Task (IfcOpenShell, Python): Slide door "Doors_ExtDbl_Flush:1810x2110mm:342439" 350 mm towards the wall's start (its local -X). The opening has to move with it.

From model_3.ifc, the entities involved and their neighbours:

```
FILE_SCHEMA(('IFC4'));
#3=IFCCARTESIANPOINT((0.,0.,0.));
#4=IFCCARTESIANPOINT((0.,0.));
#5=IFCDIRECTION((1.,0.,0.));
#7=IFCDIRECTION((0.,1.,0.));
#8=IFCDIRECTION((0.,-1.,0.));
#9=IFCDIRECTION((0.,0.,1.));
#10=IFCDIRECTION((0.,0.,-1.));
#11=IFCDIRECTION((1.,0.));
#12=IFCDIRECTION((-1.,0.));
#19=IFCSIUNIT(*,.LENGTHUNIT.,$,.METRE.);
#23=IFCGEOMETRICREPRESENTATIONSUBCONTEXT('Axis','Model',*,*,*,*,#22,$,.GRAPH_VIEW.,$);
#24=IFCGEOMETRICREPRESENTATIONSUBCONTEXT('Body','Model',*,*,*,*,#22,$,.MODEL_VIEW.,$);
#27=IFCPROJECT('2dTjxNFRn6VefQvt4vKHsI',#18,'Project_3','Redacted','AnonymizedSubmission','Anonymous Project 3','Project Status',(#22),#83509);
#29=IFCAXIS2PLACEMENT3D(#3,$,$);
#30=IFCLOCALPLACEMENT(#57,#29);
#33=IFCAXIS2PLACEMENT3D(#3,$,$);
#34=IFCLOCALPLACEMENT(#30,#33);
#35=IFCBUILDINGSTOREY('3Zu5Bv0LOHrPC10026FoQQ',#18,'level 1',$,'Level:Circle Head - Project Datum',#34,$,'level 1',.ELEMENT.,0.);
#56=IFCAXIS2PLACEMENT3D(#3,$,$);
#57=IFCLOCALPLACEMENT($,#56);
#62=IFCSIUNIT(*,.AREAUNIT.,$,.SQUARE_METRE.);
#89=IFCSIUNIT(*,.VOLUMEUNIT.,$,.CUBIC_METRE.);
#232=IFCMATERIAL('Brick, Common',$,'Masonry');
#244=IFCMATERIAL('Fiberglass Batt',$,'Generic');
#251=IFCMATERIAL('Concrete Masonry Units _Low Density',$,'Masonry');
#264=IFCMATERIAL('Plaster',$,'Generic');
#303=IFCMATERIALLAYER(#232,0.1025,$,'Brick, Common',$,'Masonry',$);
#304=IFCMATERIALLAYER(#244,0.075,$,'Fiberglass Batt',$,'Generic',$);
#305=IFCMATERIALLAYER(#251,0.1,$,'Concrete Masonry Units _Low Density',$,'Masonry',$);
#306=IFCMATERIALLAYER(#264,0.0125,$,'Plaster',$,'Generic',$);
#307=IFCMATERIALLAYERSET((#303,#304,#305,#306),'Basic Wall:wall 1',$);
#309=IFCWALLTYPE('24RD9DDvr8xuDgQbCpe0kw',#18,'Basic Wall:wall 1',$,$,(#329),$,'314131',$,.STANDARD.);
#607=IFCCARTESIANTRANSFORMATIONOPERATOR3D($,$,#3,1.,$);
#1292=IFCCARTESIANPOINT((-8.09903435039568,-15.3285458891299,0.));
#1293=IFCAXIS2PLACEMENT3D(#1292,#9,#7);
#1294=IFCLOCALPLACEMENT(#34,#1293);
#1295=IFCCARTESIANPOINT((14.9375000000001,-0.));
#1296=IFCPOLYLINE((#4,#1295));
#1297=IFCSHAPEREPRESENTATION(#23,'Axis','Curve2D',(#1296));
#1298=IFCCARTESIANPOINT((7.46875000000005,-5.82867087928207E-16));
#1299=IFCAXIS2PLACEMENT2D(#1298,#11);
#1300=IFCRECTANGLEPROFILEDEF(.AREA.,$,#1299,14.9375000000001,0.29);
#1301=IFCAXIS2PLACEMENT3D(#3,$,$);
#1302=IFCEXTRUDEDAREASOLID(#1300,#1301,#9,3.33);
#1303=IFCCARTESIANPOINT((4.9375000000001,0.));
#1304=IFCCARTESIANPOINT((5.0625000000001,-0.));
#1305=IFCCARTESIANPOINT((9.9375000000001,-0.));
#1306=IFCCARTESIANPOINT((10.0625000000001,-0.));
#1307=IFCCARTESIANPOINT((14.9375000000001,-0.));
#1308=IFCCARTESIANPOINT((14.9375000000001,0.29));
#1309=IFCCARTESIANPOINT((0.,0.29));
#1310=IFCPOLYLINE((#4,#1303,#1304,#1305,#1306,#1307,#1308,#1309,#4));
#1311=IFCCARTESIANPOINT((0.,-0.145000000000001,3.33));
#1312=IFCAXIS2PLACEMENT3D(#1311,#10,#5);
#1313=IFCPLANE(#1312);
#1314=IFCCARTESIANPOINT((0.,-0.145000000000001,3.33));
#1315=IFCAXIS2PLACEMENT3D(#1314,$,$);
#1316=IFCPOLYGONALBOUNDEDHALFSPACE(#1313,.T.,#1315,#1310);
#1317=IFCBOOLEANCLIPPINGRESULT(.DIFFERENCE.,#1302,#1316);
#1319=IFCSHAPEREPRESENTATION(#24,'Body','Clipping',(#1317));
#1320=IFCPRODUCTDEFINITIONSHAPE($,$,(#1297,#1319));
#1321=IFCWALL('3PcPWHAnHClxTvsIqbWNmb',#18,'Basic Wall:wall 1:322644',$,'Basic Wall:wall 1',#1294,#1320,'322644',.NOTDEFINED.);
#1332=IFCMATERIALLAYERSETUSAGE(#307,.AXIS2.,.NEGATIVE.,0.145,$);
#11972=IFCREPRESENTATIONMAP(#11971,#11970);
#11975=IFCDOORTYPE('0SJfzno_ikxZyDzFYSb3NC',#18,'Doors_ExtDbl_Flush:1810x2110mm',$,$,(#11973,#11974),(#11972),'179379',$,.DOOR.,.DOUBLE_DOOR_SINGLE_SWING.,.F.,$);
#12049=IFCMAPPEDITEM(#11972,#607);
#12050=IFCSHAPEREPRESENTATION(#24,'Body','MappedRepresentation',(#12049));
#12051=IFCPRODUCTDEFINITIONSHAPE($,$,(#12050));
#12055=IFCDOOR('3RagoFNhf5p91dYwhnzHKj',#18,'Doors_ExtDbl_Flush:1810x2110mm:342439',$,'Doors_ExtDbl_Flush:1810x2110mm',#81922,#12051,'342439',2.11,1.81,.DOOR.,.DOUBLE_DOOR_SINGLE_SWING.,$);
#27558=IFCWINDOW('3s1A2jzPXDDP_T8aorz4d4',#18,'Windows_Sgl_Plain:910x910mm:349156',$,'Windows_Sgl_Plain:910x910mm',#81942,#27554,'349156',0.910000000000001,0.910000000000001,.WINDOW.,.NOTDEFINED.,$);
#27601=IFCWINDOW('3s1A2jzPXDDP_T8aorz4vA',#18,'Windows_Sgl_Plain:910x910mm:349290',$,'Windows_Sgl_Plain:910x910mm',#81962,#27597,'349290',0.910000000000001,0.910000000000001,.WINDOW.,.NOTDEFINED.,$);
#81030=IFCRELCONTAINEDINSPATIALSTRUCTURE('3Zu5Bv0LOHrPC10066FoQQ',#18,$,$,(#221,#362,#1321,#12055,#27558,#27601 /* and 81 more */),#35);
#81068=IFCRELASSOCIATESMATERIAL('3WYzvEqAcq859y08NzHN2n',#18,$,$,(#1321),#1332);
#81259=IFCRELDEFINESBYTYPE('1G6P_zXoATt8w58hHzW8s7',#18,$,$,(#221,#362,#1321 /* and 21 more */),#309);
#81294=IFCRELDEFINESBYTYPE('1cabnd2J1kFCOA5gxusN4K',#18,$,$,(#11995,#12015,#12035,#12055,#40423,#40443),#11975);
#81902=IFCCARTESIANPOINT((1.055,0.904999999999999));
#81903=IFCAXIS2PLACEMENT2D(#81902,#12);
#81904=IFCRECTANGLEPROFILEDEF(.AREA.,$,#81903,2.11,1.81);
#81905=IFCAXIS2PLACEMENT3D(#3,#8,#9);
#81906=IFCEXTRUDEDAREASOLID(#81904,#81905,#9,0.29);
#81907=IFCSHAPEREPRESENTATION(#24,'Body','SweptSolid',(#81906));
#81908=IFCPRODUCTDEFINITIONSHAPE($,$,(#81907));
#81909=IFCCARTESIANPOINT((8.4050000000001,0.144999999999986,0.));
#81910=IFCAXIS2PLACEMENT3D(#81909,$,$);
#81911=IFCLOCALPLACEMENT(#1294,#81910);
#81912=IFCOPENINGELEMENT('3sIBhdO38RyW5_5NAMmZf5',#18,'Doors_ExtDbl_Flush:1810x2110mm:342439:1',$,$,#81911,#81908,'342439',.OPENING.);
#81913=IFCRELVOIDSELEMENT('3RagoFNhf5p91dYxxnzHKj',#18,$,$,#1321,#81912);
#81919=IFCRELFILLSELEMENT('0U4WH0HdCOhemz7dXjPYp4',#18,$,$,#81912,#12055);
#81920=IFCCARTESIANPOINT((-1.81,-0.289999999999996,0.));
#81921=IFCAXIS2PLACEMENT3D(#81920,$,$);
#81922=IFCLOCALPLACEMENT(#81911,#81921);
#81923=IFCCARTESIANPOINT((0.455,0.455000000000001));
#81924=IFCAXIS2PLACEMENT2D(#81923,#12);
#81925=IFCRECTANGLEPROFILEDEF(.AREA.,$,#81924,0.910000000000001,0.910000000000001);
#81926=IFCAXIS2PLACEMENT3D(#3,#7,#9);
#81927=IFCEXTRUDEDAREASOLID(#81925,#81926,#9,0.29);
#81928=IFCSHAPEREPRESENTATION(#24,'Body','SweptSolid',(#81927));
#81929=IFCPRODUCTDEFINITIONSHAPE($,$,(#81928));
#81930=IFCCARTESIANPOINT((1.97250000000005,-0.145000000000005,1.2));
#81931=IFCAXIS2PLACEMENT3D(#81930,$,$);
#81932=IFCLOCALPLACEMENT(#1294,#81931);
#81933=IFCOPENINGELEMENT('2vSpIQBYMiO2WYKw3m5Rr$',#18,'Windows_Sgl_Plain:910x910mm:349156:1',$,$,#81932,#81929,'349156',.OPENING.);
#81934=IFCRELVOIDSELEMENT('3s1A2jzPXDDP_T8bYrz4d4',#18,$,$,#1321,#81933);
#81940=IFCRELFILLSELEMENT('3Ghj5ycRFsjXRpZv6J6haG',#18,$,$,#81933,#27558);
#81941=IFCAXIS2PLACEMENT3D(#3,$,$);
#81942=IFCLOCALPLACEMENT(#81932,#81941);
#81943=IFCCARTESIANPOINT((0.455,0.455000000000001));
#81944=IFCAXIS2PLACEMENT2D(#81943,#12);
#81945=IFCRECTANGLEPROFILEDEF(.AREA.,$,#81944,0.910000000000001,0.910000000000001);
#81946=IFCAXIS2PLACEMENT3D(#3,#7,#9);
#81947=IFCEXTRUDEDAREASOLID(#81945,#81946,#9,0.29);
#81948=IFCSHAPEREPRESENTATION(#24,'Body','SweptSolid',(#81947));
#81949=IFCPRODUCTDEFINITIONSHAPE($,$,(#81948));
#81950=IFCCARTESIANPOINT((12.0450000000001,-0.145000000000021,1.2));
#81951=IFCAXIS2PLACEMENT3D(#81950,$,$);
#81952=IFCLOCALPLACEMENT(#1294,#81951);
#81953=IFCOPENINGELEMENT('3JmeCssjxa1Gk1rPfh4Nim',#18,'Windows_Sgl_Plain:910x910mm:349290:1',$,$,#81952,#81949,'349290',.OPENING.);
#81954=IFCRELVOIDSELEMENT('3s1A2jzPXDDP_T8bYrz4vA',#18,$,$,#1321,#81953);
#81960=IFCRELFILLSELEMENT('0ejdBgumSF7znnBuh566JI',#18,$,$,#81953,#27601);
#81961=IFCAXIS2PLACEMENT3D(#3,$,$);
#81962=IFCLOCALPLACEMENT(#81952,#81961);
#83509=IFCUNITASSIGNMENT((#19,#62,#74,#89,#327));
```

```python
import ifcopenshell
import ifcopenshell.api.geometry
import ifcopenshell.util.placement
import ifcopenshell.util.unit

model = ifcopenshell.open("model_3.ifc")
unit_scale = ifcopenshell.util.unit.calculate_unit_scale(model)

door = model.by_guid("3RagoFNhf5p91dYwhnzHKj")
opening = door.FillsVoids[0].RelatingOpeningElement
wall = opening.VoidsElements[0].RelatingBuildingElement

wall_matrix = ifcopenshell.util.placement.get_local_placement(wall.ObjectPlacement)
shift = wall_matrix[:3, 0] * -0.35 / unit_scale
before = ifcopenshell.util.placement.get_local_placement(door.ObjectPlacement)[:3, 3].copy()

# The door is placed relative to its opening, so it follows when the opening moves.
matrix = ifcopenshell.util.placement.get_local_placement(opening.ObjectPlacement)
matrix[:3, 3] += shift
ifcopenshell.api.geometry.edit_object_placement(
    model, product=opening, matrix=matrix, is_si=False, should_transform_children=True
)

after = ifcopenshell.util.placement.get_local_placement(door.ObjectPlacement)[:3, 3]
print("door moved by", (after - before).round(3) + 0.0)

model.write("model_3_v2.ifc")
```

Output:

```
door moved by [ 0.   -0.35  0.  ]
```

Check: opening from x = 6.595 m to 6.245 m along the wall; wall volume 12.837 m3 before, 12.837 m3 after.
